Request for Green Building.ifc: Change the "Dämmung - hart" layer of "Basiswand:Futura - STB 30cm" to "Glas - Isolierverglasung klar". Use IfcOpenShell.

First a look at what the model holds.

```python
import ifcopenshell
import ifcopenshell.util.element

model = ifcopenshell.open("Green Building.ifc")
print(model.schema)
for layer_set in model.by_type("IfcMaterialLayerSet"):
    if layer_set.LayerSetName == "Basiswand:Futura - STB 30cm":
        for layer in layer_set.MaterialLayers:
            print(layer.id(), layer.Material and layer.Material.Name, layer.LayerThickness, sep=" | ")
        print(len(ifcopenshell.util.element.get_elements_by_material(model, layer_set)), "elements and types use it")
print(sorted(m.Name for m in model.by_type("IfcMaterial") if m.Name)[:60])
```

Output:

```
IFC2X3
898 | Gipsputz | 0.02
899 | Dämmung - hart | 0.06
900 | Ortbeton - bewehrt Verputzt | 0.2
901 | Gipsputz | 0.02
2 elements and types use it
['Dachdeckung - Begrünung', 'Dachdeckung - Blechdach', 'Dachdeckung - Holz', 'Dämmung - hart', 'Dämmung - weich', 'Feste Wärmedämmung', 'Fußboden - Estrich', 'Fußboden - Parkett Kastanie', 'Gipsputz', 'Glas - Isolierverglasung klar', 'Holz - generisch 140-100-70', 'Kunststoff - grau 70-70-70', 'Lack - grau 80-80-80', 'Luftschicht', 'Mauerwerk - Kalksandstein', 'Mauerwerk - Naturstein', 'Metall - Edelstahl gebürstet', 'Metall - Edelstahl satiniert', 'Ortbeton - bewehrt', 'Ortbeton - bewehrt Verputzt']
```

```python
import ifcopenshell
import ifcopenshell.api.material

model = ifcopenshell.open("Green Building.ifc")

layer_set = next(s for s in model.by_type("IfcMaterialLayerSet") if s.LayerSetName == "Basiswand:Futura - STB 30cm")
layer = next(l for l in layer_set.MaterialLayers if l.Material and l.Material.Name == "Dämmung - hart")
material = next(m for m in model.by_type("IfcMaterial") if m.Name == "Glas - Isolierverglasung klar")

# Point this one layer at the other material; renaming the old one would change it everywhere.
ifcopenshell.api.material.edit_layer(model, layer=layer, attributes={}, material=material)

print([l.Material.Name if l.Material else None for l in layer_set.MaterialLayers])

model.write("Green Building_v2.ifc")
```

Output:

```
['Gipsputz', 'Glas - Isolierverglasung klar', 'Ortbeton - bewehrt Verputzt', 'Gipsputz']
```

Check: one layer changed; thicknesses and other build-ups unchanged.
